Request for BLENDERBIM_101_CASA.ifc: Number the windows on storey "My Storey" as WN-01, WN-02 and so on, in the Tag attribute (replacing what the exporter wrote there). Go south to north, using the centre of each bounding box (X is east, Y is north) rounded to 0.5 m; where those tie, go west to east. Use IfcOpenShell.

First a look at what the model holds.

```python
import ifcopenshell
import ifcopenshell.util.element
import ifcopenshell.util.placement

model = ifcopenshell.open("BLENDERBIM_101_CASA.ifc")
print(model.schema)
storey = next(s for s in model.by_type("IfcBuildingStorey") if s.Name == "My Storey")
windows = [e for e in ifcopenshell.util.element.get_decomposition(storey) if e.is_a("IfcWindow")]
for e in sorted(windows, key=lambda e: e.id()):
    origin = ifcopenshell.util.placement.get_local_placement(e.ObjectPlacement)[:3, 3]
    print(e.id(), e.Tag, e.Name, origin.round(2) + 0.0, sep=" | ")
```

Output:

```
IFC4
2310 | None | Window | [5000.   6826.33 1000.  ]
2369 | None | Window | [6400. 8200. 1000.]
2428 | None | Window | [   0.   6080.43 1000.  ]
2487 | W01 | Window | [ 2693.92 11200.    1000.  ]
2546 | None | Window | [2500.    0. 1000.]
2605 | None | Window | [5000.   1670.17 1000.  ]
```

```python
import ifcopenshell
import ifcopenshell.geom
import ifcopenshell.util.element
import ifcopenshell.util.shape

model = ifcopenshell.open("BLENDERBIM_101_CASA.ifc")
settings = ifcopenshell.geom.settings()
settings.set("use-world-coords", True)


def centre(element):
    shape = ifcopenshell.geom.create_shape(settings, element)
    return ifcopenshell.util.shape.get_bbox_centroid(shape.geometry)


storey = next(s for s in model.by_type("IfcBuildingStorey") if s.Name == "My Storey")
windows = [e for e in ifcopenshell.util.element.get_decomposition(storey) if e.is_a("IfcWindow")]

# Insertion points can sit at a corner or the storey origin, so sort by the geometry (in metres).
centres = {e: centre(e) for e in windows}
windows.sort(key=lambda e: (round(centres[e][1] / 0.5), centres[e][0]))

for i, e in enumerate(windows, start=1):
    number = f"WN-{i:02d}"
    e.Tag = number
    print(e.id(), number)

model.write("BLENDERBIM_101_CASA_updated.ifc")
```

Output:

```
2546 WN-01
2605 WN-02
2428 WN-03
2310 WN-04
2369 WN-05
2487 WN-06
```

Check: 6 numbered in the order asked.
